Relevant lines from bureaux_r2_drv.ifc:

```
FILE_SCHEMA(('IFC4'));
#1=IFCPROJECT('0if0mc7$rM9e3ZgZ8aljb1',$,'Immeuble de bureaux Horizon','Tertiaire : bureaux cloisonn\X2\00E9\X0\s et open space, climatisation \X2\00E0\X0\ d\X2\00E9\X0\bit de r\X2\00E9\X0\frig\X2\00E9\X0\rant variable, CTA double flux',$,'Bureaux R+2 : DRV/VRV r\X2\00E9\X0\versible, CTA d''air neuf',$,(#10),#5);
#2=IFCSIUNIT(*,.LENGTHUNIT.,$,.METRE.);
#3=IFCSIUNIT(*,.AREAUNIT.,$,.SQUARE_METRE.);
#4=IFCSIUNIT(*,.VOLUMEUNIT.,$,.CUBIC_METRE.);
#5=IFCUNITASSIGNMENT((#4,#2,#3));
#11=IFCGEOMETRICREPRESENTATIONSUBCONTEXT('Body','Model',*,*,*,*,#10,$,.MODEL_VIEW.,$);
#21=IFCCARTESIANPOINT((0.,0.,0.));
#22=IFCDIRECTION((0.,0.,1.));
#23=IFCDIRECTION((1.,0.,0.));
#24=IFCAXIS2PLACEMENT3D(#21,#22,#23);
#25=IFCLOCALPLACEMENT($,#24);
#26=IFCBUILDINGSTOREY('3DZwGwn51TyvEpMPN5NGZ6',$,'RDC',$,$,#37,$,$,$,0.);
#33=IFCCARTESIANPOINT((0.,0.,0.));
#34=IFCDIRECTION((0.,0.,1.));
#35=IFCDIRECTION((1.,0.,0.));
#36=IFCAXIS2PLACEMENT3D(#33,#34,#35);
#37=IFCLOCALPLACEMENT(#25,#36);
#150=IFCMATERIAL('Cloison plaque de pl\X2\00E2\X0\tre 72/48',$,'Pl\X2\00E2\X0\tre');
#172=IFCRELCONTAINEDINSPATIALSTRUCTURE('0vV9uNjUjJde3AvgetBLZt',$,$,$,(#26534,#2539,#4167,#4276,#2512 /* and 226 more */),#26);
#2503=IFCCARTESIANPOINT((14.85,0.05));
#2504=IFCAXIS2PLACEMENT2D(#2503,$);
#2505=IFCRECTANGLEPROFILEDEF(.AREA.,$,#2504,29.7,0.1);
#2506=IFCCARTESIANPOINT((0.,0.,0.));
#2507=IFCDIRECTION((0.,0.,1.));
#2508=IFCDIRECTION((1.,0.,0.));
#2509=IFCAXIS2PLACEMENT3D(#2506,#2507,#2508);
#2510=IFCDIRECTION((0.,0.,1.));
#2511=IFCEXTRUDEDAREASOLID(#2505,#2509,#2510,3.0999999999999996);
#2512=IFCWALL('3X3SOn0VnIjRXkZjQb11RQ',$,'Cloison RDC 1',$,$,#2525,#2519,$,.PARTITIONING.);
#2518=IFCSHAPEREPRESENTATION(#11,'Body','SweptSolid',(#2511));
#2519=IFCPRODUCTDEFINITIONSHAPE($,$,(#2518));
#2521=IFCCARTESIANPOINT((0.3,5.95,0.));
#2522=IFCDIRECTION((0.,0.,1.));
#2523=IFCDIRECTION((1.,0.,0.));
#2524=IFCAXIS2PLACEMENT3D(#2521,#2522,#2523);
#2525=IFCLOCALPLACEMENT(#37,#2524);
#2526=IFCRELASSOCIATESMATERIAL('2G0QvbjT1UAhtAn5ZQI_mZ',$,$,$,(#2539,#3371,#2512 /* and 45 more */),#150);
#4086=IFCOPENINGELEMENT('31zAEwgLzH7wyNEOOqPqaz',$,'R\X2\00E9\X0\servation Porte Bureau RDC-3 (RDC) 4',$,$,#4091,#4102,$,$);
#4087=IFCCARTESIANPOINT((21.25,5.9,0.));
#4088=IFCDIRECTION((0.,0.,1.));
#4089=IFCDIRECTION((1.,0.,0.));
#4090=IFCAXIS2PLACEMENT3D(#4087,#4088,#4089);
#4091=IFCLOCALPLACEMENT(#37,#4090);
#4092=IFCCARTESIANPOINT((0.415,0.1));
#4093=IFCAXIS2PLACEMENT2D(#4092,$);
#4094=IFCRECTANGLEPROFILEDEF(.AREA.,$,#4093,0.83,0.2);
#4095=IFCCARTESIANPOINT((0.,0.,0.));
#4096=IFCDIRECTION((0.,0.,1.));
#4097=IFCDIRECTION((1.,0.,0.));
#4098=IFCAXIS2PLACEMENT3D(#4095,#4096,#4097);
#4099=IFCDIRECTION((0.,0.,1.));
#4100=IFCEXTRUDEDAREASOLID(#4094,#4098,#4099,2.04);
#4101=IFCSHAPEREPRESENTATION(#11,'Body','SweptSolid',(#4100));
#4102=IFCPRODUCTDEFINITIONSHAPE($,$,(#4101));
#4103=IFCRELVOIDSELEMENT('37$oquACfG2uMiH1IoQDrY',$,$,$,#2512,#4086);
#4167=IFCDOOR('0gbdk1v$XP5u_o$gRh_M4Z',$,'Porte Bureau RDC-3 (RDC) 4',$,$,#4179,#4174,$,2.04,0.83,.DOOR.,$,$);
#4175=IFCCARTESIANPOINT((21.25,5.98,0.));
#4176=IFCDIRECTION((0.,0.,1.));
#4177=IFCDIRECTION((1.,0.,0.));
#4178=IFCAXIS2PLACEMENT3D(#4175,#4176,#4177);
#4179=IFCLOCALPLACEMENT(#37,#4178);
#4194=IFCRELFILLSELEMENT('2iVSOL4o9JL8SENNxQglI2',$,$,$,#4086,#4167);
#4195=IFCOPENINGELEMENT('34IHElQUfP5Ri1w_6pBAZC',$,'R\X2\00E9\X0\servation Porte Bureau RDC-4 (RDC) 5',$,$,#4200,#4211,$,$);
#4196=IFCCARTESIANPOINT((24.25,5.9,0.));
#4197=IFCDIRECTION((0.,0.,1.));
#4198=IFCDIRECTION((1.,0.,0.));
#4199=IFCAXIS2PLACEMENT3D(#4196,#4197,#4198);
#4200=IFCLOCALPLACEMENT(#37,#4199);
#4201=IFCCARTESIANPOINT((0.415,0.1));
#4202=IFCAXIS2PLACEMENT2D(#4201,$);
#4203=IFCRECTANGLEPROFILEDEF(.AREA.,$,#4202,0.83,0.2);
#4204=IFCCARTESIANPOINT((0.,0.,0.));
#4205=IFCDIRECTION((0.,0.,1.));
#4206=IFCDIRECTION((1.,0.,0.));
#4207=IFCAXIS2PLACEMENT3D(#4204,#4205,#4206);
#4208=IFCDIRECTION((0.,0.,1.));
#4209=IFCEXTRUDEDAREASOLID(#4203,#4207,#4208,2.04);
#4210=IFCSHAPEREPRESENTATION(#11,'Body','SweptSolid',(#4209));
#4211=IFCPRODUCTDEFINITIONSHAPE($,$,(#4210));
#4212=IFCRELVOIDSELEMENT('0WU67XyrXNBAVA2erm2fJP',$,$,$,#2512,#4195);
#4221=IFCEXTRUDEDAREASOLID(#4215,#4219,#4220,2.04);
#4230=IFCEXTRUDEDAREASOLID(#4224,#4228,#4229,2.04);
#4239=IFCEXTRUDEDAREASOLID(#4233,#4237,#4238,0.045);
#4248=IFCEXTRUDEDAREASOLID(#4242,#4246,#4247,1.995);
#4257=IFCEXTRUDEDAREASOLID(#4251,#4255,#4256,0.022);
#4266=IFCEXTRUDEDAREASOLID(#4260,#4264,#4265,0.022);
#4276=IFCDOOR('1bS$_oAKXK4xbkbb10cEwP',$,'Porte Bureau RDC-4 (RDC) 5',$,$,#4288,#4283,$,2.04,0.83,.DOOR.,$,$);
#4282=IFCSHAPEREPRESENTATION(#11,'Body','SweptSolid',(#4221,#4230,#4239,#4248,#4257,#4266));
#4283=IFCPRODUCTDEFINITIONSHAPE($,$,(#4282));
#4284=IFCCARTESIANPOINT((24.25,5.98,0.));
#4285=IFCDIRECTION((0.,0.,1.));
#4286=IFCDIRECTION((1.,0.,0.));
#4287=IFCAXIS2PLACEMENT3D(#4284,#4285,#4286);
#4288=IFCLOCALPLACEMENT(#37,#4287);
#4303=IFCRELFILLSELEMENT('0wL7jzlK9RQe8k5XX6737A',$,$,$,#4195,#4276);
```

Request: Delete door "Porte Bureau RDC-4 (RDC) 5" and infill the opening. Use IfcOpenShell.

```python
import ifcopenshell
import ifcopenshell.api.feature
import ifcopenshell.api.root
import ifcopenshell.geom
import ifcopenshell.util.shape

model = ifcopenshell.open("bureaux_r2_drv.ifc")
settings = ifcopenshell.geom.settings()


def volume(element):
    """Net volume in cubic metres, openings subtracted."""
    shape = ifcopenshell.geom.create_shape(settings, element)
    return ifcopenshell.util.shape.get_volume(shape.geometry)


door = model.by_guid("1bS$_oAKXK4xbkbb10cEwP")
opening = door.FillsVoids[0].RelatingOpeningElement
wall = opening.VoidsElements[0].RelatingBuildingElement
before = volume(wall)

ifcopenshell.api.root.remove_product(model, product=door)
ifcopenshell.api.feature.remove_feature(model, feature=opening)

after = volume(wall)

print(f"wall volume {before:.3f} -> {after:.3f} m3")

model.write("bureaux_r2_drv_edited.ifc")
```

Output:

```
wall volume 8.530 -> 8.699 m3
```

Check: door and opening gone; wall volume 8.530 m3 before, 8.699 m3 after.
